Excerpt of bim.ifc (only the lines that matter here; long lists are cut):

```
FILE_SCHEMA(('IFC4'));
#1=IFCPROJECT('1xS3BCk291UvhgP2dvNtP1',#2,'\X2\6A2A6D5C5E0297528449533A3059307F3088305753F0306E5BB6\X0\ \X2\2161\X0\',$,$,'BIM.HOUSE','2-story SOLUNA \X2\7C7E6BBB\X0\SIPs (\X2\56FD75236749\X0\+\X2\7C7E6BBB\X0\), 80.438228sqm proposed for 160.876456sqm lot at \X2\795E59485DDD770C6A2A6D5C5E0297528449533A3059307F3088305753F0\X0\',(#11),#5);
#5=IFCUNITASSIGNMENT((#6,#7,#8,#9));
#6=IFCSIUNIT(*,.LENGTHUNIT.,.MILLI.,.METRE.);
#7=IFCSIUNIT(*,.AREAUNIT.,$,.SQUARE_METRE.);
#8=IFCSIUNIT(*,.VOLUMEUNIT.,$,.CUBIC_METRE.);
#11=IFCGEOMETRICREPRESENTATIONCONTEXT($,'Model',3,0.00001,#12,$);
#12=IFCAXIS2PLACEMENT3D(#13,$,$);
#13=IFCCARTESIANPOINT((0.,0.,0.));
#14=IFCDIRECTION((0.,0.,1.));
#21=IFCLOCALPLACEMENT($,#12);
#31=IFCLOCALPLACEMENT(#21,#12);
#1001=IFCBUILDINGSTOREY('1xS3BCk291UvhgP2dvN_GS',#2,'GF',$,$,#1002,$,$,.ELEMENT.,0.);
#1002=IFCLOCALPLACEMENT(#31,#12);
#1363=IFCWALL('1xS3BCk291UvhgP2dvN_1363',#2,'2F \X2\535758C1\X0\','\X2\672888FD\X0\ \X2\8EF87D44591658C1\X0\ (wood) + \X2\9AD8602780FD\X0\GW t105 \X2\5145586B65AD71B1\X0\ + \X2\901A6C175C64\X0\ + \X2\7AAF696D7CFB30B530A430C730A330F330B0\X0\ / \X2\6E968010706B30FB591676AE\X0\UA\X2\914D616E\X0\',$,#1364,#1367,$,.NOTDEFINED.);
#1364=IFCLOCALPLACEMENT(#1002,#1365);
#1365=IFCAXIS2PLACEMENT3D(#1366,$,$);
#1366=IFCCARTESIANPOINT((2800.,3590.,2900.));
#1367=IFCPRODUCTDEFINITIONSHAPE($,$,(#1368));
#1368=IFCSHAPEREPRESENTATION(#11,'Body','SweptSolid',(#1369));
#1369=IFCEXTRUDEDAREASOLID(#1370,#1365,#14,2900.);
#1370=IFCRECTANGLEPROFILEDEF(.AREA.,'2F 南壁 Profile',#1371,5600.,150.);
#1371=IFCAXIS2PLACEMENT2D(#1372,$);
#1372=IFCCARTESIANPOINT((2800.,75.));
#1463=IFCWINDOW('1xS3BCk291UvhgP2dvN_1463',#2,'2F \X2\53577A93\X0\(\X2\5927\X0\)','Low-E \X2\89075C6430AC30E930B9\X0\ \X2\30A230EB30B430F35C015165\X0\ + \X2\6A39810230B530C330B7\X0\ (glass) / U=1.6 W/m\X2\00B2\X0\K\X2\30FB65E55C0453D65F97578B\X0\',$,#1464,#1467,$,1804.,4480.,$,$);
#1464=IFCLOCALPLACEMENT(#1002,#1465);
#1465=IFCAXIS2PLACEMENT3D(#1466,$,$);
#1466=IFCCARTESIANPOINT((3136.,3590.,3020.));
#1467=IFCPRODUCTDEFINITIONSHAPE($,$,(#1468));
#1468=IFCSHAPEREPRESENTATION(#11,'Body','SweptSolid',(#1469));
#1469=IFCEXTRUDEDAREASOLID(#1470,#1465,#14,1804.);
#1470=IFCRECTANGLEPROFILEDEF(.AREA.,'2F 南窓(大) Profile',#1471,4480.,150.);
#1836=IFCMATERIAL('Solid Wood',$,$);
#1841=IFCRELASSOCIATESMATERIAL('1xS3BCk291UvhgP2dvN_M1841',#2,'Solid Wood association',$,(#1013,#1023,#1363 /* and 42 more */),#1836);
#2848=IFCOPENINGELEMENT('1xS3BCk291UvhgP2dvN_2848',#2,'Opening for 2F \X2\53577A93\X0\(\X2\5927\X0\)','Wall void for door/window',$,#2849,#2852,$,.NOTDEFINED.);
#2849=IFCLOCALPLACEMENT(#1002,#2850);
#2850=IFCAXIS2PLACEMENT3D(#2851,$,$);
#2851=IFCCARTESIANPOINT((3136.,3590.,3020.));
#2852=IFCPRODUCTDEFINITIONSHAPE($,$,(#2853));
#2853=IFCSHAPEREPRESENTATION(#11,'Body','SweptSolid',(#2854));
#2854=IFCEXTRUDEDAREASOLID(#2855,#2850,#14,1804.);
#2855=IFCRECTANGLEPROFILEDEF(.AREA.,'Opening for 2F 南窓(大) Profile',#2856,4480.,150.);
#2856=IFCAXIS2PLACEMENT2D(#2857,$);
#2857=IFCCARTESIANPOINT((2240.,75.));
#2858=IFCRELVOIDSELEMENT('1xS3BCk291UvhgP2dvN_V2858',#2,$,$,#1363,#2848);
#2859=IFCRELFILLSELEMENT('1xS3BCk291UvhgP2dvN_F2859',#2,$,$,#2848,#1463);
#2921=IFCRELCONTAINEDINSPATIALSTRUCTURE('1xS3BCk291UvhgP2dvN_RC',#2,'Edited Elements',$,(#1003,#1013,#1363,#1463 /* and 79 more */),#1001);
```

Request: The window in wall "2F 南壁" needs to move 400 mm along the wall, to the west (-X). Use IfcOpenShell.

```python
import ifcopenshell
import ifcopenshell.api.geometry
import ifcopenshell.util.placement
import ifcopenshell.util.unit

model = ifcopenshell.open("bim.ifc")
unit_scale = ifcopenshell.util.unit.calculate_unit_scale(model)

window = model.by_guid("1xS3BCk291UvhgP2dvN_1463")
opening = window.FillsVoids[0].RelatingOpeningElement
wall = opening.VoidsElements[0].RelatingBuildingElement

wall_matrix = ifcopenshell.util.placement.get_local_placement(wall.ObjectPlacement)
shift = wall_matrix[:3, 0] * -0.4 / unit_scale
before = ifcopenshell.util.placement.get_local_placement(window.ObjectPlacement)[:3, 3].copy()

# The window is not placed relative to its opening, so move both.
for product in (opening, window):
    matrix = ifcopenshell.util.placement.get_local_placement(product.ObjectPlacement)
    matrix[:3, 3] += shift
    ifcopenshell.api.geometry.edit_object_placement(model, product=product, matrix=matrix, is_si=False)

after = ifcopenshell.util.placement.get_local_placement(window.ObjectPlacement)[:3, 3]
print("window moved by", (after - before).round(3) + 0.0)

model.write("bim_rev.ifc")
```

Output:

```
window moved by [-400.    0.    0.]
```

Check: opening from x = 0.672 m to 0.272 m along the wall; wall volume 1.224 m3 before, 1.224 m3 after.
